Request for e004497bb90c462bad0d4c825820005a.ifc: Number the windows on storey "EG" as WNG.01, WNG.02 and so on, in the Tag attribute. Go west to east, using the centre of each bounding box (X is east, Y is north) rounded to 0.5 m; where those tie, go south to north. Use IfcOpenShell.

First a look at what the model holds.

```python
import ifcopenshell
import ifcopenshell.util.element
import ifcopenshell.util.placement

model = ifcopenshell.open("e004497bb90c462bad0d4c825820005a.ifc")
print(model.schema)
storey = next(s for s in model.by_type("IfcBuildingStorey") if s.Name == "EG")
windows = [e for e in ifcopenshell.util.element.get_decomposition(storey) if e.is_a("IfcWindow")]
for e in sorted(windows, key=lambda e: e.id()):
    origin = ifcopenshell.util.placement.get_local_placement(e.ObjectPlacement)[:3, 3]
    print(e.id(), e.Tag, e.Name, origin.round(2) + 0.0, sep=" | ")
```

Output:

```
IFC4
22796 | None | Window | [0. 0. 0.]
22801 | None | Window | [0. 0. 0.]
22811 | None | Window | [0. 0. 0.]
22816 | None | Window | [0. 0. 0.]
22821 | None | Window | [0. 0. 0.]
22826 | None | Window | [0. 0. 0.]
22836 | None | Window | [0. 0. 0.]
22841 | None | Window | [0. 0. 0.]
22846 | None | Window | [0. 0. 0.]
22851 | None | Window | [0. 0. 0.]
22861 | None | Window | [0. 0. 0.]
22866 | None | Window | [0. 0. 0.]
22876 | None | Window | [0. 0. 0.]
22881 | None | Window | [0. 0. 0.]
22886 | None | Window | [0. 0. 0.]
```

```python
import ifcopenshell
import ifcopenshell.geom
import ifcopenshell.util.element
import ifcopenshell.util.shape

model = ifcopenshell.open("e004497bb90c462bad0d4c825820005a.ifc")
settings = ifcopenshell.geom.settings()
settings.set("use-world-coords", True)


def centre(element):
    shape = ifcopenshell.geom.create_shape(settings, element)
    return ifcopenshell.util.shape.get_bbox_centroid(shape.geometry)


storey = next(s for s in model.by_type("IfcBuildingStorey") if s.Name == "EG")
windows = [e for e in ifcopenshell.util.element.get_decomposition(storey) if e.is_a("IfcWindow")]

# Insertion points can sit at a corner or the storey origin, so sort by the geometry (in metres).
centres = {e: centre(e) for e in windows}
windows.sort(key=lambda e: (round(centres[e][0] / 0.5), centres[e][1]))

for i, e in enumerate(windows, start=1):
    number = f"WNG.{i:02d}"
    e.Tag = number
    print(e.id(), number)

model.write("e004497bb90c462bad0d4c825820005a_rev.ifc")
```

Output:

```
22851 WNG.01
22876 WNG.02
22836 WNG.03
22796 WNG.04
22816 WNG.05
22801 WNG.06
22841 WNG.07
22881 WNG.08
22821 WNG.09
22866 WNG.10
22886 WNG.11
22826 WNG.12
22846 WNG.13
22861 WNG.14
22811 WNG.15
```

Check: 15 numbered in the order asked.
